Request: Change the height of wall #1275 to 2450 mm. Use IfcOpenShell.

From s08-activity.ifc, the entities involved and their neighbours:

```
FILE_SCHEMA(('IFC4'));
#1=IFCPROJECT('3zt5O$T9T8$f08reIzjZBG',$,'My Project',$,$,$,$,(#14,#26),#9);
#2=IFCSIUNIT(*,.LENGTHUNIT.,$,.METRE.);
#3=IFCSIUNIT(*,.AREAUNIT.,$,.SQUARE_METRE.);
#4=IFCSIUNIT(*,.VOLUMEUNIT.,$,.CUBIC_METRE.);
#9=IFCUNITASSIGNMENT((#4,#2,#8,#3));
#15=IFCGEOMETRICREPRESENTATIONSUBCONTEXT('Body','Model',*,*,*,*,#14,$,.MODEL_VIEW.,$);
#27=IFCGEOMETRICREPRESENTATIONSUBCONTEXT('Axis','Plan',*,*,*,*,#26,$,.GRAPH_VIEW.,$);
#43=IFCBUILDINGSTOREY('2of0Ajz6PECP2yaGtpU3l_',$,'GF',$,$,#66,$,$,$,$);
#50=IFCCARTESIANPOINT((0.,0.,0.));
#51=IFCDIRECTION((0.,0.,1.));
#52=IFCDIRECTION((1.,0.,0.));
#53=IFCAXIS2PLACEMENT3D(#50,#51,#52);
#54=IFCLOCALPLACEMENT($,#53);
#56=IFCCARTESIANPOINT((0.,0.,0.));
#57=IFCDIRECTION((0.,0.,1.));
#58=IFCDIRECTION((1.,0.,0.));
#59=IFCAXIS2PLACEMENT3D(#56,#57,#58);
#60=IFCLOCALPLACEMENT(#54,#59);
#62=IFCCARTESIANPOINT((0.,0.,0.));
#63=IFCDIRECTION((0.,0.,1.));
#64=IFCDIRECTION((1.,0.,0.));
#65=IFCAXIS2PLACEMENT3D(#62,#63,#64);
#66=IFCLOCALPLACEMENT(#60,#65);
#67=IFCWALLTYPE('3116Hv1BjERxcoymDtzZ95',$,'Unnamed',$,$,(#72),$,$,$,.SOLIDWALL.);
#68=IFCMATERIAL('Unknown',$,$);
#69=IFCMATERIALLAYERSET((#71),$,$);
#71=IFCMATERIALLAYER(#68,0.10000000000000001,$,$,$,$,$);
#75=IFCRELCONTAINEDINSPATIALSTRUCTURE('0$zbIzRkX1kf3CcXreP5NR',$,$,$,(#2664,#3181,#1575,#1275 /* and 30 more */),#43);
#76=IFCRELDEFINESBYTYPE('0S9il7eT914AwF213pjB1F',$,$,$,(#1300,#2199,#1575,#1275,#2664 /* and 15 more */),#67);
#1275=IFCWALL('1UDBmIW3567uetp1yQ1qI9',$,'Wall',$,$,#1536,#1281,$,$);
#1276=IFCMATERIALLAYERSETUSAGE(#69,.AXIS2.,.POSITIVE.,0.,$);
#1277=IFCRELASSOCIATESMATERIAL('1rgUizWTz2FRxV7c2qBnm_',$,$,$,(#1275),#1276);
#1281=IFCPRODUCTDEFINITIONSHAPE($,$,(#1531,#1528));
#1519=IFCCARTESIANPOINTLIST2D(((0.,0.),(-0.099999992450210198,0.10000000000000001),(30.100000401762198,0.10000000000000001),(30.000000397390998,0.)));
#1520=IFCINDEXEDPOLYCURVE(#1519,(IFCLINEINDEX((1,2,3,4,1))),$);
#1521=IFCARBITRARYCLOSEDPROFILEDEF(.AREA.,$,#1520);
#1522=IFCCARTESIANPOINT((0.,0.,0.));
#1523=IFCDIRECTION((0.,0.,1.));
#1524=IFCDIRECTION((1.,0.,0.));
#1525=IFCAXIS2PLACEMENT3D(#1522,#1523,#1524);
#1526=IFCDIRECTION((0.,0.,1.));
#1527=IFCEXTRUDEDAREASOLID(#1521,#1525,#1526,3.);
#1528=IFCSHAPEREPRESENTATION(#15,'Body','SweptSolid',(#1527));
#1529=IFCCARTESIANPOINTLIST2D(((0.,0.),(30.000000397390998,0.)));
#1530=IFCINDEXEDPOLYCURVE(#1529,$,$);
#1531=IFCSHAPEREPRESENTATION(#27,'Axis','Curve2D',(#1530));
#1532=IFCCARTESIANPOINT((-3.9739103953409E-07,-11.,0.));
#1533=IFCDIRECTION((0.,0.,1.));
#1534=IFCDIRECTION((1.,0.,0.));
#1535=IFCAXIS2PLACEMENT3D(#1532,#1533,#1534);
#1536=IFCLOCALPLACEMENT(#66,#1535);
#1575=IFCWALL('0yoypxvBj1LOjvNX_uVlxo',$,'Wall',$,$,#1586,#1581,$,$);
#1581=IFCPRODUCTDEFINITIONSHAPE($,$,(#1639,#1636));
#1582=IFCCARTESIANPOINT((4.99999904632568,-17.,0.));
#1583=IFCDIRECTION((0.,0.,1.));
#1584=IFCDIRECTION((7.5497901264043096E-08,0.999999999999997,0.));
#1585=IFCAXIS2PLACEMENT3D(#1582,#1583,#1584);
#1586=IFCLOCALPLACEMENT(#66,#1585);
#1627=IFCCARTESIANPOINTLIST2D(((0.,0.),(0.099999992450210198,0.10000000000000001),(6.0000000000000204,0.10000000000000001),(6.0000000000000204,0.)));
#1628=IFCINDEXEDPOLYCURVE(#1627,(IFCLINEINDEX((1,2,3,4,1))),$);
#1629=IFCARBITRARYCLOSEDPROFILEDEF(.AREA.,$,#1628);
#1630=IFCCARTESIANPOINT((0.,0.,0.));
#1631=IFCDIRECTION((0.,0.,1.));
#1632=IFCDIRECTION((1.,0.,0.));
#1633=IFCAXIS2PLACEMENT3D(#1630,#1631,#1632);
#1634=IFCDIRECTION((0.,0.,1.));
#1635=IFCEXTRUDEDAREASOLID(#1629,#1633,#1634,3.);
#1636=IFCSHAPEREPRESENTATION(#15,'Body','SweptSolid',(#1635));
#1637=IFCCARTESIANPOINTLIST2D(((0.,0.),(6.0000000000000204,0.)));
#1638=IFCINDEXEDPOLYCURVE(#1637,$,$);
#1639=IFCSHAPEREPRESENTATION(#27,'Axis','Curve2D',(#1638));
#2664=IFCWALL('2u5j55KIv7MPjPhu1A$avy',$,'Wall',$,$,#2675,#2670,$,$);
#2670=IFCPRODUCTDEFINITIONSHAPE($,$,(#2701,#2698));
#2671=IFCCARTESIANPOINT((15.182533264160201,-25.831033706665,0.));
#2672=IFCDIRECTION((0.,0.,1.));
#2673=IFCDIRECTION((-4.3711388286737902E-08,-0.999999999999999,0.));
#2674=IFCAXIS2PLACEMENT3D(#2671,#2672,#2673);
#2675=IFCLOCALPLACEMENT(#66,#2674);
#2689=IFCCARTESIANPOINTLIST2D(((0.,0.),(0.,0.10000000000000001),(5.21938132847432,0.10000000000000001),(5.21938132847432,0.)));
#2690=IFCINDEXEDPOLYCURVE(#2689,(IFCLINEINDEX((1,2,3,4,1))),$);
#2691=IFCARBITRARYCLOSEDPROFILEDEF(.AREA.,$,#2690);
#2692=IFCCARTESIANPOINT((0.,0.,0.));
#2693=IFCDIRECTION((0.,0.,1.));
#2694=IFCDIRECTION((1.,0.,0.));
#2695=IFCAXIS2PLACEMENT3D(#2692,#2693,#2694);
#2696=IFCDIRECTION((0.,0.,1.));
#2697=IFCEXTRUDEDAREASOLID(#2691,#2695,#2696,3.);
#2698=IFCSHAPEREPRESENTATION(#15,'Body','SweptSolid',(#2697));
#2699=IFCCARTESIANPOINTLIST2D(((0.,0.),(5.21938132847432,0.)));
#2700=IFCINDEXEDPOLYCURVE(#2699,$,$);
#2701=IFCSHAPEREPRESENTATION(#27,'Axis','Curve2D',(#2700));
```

```python
import ifcopenshell
import ifcopenshell.geom
import ifcopenshell.util.representation
import ifcopenshell.util.shape
import ifcopenshell.util.unit

model = ifcopenshell.open("s08-activity.ifc")
unit_scale = ifcopenshell.util.unit.calculate_unit_scale(model)
settings = ifcopenshell.geom.settings()


def volume(element):
    """Net volume in cubic metres, openings subtracted."""
    shape = ifcopenshell.geom.create_shape(settings, element)
    return ifcopenshell.util.shape.get_volume(shape.geometry)


wall = model.by_id(1275)
before = volume(wall)

body = ifcopenshell.util.representation.get_representation(wall, "Model", "Body")
solid = body.Items[0]
old_height = solid.Depth
solid.Depth = 2.45 / unit_scale
after = volume(wall)

print(f"height {old_height:g} -> {solid.Depth:g}, volume {before:.3f} -> {after:.3f} m3")

model.write("s08-activity-out.ifc")
```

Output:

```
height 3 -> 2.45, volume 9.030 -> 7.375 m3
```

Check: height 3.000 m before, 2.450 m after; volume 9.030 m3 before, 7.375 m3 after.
